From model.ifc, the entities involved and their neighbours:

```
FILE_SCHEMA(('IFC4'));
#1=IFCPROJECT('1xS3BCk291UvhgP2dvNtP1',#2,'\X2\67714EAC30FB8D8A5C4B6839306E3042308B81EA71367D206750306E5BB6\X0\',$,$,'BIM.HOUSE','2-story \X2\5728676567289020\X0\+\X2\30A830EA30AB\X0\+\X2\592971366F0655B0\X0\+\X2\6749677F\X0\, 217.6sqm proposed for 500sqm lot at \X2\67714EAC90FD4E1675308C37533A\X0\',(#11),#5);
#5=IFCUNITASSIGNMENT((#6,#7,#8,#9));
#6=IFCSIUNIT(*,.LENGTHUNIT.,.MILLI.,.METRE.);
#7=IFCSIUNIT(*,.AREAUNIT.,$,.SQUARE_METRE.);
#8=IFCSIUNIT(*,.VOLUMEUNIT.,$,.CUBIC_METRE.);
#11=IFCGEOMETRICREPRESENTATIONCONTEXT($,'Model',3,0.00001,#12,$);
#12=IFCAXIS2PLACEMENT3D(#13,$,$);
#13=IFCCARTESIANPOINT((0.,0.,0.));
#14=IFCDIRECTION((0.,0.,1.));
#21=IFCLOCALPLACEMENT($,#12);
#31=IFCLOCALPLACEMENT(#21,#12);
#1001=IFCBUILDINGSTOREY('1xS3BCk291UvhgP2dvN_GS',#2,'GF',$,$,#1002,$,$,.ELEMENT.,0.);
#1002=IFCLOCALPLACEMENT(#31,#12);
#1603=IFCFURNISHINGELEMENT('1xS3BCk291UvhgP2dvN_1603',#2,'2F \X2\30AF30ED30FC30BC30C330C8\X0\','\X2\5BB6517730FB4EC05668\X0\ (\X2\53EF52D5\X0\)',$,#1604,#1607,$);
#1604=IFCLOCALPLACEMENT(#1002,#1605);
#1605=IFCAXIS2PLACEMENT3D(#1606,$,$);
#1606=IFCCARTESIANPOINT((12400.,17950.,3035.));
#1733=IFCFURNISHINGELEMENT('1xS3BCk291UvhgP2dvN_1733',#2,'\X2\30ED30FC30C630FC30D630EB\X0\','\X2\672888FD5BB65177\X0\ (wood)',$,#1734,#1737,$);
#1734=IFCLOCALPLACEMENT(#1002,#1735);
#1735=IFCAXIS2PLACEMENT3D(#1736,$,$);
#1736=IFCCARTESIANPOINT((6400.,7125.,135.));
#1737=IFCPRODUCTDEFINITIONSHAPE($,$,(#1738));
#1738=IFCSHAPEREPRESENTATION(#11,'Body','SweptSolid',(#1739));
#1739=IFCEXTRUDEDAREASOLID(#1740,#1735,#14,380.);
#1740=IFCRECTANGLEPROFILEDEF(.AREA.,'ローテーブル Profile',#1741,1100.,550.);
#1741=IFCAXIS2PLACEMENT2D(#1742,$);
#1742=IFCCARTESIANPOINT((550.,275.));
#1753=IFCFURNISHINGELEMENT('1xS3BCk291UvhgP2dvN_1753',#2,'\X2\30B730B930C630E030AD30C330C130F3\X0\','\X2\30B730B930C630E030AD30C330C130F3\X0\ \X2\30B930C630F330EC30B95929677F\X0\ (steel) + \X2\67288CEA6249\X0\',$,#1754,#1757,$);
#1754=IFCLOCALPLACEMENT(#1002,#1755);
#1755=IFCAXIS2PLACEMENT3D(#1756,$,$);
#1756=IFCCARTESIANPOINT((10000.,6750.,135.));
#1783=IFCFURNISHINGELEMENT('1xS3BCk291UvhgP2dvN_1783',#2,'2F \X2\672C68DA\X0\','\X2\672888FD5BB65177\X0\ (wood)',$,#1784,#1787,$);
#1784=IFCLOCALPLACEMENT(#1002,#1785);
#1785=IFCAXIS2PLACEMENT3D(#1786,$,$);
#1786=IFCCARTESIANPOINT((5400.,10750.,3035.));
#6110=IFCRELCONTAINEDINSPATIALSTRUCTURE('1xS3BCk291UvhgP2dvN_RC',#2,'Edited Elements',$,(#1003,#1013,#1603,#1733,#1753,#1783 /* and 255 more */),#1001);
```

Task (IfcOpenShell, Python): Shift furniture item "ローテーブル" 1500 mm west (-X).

```python
import ifcopenshell
import ifcopenshell.api.geometry
import ifcopenshell.util.placement
import ifcopenshell.util.unit

model = ifcopenshell.open("model.ifc")
unit_scale = ifcopenshell.util.unit.calculate_unit_scale(model)

item = model.by_id(1733)
matrix = ifcopenshell.util.placement.get_local_placement(item.ObjectPlacement)
matrix[0, 3] -= 1.5 / unit_scale
ifcopenshell.api.geometry.edit_object_placement(model, product=item, matrix=matrix, is_si=False)

print(ifcopenshell.util.placement.get_local_placement(item.ObjectPlacement).round(3) + 0.0)

model.write("model_edited.ifc")
```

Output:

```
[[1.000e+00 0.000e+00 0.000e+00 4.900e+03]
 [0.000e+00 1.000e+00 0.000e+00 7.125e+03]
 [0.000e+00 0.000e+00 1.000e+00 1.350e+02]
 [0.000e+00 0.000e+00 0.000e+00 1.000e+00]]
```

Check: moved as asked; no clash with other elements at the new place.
